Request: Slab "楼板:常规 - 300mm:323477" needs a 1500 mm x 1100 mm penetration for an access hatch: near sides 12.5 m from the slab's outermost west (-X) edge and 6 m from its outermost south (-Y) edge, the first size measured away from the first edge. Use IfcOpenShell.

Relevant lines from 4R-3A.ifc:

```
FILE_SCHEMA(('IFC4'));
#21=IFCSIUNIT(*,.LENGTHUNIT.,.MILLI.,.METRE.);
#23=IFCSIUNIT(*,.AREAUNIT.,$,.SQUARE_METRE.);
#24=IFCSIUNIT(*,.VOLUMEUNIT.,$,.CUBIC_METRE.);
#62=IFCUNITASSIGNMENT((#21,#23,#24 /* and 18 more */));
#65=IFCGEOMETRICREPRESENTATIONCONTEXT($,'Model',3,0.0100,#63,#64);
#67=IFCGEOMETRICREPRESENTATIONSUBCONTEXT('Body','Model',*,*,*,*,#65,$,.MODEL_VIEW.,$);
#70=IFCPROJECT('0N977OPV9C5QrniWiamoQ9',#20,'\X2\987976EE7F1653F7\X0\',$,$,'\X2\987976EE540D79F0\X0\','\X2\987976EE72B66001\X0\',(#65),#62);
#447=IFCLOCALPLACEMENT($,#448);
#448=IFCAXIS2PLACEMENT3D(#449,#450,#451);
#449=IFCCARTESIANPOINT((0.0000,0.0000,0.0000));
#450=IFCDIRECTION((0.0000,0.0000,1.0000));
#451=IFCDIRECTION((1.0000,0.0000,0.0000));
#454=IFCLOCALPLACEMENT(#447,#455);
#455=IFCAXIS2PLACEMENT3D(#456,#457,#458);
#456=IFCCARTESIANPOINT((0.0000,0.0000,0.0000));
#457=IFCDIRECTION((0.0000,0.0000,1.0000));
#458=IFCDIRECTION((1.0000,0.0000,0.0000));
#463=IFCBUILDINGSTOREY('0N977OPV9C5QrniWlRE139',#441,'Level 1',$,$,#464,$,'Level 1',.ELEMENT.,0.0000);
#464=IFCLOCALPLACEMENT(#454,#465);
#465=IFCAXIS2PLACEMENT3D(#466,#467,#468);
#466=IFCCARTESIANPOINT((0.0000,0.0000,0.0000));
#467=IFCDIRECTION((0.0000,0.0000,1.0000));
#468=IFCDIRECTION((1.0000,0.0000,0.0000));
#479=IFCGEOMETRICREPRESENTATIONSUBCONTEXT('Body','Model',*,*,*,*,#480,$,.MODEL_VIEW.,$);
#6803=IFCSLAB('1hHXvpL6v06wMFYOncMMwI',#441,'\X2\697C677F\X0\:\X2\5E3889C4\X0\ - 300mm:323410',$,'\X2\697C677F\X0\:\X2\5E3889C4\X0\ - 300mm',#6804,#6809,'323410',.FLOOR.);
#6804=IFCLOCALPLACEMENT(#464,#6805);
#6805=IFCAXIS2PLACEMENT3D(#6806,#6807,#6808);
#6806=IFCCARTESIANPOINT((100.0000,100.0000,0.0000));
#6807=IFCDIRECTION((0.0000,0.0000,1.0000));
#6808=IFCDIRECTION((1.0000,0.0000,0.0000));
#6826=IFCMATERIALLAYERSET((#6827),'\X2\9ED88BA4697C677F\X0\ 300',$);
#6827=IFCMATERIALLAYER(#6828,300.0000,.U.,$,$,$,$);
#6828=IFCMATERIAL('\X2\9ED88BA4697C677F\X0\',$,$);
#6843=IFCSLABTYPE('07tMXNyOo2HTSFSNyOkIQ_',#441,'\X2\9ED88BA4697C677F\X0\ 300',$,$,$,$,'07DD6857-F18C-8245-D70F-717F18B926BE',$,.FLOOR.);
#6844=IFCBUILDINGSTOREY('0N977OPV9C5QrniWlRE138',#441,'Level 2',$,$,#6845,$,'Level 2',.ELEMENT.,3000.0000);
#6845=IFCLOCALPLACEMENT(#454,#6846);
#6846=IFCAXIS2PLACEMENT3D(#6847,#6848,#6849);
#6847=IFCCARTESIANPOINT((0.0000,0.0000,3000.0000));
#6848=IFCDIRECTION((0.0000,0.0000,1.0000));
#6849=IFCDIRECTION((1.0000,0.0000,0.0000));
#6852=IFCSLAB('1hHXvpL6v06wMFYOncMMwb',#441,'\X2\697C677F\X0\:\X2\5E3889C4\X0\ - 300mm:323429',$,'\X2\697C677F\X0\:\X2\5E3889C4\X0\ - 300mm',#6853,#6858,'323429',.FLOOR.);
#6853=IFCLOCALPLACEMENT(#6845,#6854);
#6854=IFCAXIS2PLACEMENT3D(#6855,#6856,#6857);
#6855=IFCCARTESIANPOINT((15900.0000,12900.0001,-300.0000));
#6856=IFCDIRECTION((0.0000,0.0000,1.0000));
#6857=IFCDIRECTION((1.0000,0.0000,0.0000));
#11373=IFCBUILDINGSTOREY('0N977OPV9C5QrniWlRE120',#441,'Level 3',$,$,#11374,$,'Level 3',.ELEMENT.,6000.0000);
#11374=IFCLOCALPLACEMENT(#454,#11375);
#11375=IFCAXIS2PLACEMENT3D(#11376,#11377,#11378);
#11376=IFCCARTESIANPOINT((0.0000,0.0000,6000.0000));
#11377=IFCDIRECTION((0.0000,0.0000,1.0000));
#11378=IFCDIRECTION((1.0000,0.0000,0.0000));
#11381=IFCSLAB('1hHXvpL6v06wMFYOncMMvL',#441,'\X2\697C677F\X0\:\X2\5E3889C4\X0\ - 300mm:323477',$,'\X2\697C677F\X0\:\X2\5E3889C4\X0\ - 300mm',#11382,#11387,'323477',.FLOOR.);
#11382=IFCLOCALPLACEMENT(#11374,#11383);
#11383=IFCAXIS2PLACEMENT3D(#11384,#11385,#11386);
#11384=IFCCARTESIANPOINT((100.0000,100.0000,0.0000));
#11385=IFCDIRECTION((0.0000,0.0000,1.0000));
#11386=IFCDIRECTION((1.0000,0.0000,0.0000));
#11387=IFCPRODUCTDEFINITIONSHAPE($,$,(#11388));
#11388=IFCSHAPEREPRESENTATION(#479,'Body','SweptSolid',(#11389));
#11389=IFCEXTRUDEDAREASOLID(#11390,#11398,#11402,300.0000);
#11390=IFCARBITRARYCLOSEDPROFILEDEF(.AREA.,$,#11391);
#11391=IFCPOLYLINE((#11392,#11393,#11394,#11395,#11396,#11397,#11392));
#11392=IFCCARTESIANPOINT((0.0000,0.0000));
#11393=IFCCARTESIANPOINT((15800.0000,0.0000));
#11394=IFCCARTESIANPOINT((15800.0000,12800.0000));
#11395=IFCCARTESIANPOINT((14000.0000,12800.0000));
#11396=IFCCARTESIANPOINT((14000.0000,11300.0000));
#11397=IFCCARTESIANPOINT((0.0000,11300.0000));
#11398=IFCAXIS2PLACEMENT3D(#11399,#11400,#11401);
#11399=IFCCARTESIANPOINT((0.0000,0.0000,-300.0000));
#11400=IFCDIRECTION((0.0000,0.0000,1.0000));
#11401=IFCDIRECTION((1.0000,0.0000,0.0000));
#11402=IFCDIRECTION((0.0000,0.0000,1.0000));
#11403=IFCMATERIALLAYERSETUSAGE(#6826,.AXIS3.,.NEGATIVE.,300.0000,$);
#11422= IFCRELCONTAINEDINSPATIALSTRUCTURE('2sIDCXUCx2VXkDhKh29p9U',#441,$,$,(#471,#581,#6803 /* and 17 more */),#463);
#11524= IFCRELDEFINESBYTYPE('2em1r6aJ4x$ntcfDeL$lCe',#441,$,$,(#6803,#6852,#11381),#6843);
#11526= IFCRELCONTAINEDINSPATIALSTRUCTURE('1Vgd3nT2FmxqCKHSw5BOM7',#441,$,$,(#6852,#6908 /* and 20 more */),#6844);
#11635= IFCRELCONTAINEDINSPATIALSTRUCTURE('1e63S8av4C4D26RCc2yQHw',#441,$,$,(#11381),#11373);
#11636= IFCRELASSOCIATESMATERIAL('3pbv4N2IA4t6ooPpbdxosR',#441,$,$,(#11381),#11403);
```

```python
import numpy as np
import ifcopenshell
import ifcopenshell.api.feature
import ifcopenshell.api.geometry
import ifcopenshell.api.root
import ifcopenshell.geom
import ifcopenshell.util.placement
import ifcopenshell.util.representation
import ifcopenshell.util.shape
import ifcopenshell.util.unit

model = ifcopenshell.open("4R-3A.ifc")
unit_scale = ifcopenshell.util.unit.calculate_unit_scale(model)
settings = ifcopenshell.geom.settings()


def volume(element):
    """Net volume in cubic metres, openings subtracted."""
    shape = ifcopenshell.geom.create_shape(settings, element)
    return ifcopenshell.util.shape.get_volume(shape.geometry)


slab = model.by_id(11381)
before = volume(slab)

# Extent in the slab's own axes, in metres. The edges named are its -X and -Y sides.
slab_shape = ifcopenshell.geom.create_shape(settings, slab)
vertices = ifcopenshell.util.shape.get_vertices(slab_shape.geometry)
x_min, y_min, bottom = vertices.min(axis=0)
top = vertices[:, 2].max()

opening = ifcopenshell.api.root.create_entity(model, ifc_class="IfcOpeningElement", name="Access hatch opening", predefined_type="OPENING")
context = ifcopenshell.util.representation.get_context(model, "Model", "Body", "MODEL_VIEW")
width, depth = 1.5, 1.1
outline = [(0.0, 0.0), (width, 0.0), (width, depth), (0.0, depth), (0.0, 0.0)]
# Overshoot both faces by 50 mm so the cut is clean.
shape = ifcopenshell.api.geometry.add_slab_representation(
    model, context=context, depth=top - bottom + 0.1, polyline=outline
)
ifcopenshell.api.geometry.assign_representation(model, product=opening, representation=shape)

matrix = ifcopenshell.util.placement.get_local_placement(slab.ObjectPlacement)
matrix[:, 3] = matrix @ np.append(np.array([x_min + 12.5, y_min + 6, bottom - 0.05]) / unit_scale, 1.0)
ifcopenshell.api.geometry.edit_object_placement(model, product=opening, matrix=matrix, is_si=False)
ifcopenshell.api.feature.add_feature(model, feature=opening, element=slab)

after = volume(slab)

print(f"slab volume {before:.3f} -> {after:.3f} m3")

model.write("4R-3A_v2.ifc")
```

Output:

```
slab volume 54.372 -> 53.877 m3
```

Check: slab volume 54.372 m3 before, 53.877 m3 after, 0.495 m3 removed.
